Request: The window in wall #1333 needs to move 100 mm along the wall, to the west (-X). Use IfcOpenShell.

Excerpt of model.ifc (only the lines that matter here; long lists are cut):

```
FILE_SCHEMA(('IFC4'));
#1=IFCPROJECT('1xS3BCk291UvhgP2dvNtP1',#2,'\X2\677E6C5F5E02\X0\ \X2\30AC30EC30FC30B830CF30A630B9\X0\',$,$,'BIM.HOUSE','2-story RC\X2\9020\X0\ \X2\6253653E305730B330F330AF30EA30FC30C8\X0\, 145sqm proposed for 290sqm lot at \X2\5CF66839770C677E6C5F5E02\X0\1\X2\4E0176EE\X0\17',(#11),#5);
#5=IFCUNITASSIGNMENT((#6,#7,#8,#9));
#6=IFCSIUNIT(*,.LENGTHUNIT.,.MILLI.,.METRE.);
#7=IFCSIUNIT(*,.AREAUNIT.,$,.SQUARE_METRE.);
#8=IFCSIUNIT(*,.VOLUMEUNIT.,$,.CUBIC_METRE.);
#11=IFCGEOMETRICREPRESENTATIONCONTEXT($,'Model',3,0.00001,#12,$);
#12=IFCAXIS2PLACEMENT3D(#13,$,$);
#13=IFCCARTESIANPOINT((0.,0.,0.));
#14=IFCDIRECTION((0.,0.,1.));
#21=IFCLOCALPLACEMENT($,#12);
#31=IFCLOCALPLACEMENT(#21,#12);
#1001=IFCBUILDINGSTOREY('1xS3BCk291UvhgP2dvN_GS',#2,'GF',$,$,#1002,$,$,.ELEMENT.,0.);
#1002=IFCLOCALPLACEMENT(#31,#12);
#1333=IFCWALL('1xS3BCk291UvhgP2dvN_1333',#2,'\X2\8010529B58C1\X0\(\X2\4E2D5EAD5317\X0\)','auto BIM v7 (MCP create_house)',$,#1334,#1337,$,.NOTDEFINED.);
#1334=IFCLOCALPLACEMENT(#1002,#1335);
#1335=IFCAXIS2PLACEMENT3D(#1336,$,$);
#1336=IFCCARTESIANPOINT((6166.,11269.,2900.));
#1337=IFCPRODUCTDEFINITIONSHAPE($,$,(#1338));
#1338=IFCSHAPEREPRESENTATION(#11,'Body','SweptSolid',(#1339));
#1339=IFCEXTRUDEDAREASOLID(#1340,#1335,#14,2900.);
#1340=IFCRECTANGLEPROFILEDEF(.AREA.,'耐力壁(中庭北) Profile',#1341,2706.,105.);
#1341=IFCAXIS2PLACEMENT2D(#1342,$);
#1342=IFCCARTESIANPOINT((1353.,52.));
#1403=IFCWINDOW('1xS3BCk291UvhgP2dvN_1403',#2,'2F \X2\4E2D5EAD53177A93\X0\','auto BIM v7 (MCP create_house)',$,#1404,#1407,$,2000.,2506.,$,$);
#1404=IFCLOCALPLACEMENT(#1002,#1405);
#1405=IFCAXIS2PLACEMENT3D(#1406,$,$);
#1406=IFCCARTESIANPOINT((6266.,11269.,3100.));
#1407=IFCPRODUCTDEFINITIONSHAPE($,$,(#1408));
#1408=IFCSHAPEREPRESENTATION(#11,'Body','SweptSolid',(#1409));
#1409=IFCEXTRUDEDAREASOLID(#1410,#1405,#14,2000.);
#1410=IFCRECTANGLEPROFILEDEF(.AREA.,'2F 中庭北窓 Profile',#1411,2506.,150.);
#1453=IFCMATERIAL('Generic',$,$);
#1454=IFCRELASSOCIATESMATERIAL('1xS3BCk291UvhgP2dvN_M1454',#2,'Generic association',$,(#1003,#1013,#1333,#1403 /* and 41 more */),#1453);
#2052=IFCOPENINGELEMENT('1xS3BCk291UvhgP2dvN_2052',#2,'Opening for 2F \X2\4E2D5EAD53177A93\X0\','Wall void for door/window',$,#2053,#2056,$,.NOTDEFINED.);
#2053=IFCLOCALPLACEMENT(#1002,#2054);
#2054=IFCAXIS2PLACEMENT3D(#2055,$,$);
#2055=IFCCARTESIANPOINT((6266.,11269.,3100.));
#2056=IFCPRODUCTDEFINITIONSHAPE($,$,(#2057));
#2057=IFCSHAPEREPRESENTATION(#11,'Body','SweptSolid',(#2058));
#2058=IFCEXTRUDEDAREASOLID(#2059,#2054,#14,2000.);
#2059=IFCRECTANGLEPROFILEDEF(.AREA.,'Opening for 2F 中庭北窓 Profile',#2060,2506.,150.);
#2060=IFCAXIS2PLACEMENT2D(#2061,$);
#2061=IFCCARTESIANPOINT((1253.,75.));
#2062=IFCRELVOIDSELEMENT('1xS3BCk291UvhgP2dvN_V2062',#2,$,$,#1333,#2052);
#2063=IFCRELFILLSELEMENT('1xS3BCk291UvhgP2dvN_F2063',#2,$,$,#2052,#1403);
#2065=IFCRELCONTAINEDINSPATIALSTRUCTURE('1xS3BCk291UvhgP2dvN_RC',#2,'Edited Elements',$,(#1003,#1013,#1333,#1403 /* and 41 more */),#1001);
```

```python
import ifcopenshell
import ifcopenshell.api.geometry
import ifcopenshell.util.placement
import ifcopenshell.util.unit

model = ifcopenshell.open("model.ifc")
unit_scale = ifcopenshell.util.unit.calculate_unit_scale(model)

window = model.by_guid("1xS3BCk291UvhgP2dvN_1403")
opening = window.FillsVoids[0].RelatingOpeningElement
wall = opening.VoidsElements[0].RelatingBuildingElement

wall_matrix = ifcopenshell.util.placement.get_local_placement(wall.ObjectPlacement)
shift = wall_matrix[:3, 0] * -0.1 / unit_scale
before = ifcopenshell.util.placement.get_local_placement(window.ObjectPlacement)[:3, 3].copy()

# The window is not placed relative to its opening, so move both.
for product in (opening, window):
    matrix = ifcopenshell.util.placement.get_local_placement(product.ObjectPlacement)
    matrix[:3, 3] += shift
    ifcopenshell.api.geometry.edit_object_placement(model, product=product, matrix=matrix, is_si=False)

after = ifcopenshell.util.placement.get_local_placement(window.ObjectPlacement)[:3, 3]
print("window moved by", (after - before).round(3) + 0.0)

model.write("model_updated.ifc")
```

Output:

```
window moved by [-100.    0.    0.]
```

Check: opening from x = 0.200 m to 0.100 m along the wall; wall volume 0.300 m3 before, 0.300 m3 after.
